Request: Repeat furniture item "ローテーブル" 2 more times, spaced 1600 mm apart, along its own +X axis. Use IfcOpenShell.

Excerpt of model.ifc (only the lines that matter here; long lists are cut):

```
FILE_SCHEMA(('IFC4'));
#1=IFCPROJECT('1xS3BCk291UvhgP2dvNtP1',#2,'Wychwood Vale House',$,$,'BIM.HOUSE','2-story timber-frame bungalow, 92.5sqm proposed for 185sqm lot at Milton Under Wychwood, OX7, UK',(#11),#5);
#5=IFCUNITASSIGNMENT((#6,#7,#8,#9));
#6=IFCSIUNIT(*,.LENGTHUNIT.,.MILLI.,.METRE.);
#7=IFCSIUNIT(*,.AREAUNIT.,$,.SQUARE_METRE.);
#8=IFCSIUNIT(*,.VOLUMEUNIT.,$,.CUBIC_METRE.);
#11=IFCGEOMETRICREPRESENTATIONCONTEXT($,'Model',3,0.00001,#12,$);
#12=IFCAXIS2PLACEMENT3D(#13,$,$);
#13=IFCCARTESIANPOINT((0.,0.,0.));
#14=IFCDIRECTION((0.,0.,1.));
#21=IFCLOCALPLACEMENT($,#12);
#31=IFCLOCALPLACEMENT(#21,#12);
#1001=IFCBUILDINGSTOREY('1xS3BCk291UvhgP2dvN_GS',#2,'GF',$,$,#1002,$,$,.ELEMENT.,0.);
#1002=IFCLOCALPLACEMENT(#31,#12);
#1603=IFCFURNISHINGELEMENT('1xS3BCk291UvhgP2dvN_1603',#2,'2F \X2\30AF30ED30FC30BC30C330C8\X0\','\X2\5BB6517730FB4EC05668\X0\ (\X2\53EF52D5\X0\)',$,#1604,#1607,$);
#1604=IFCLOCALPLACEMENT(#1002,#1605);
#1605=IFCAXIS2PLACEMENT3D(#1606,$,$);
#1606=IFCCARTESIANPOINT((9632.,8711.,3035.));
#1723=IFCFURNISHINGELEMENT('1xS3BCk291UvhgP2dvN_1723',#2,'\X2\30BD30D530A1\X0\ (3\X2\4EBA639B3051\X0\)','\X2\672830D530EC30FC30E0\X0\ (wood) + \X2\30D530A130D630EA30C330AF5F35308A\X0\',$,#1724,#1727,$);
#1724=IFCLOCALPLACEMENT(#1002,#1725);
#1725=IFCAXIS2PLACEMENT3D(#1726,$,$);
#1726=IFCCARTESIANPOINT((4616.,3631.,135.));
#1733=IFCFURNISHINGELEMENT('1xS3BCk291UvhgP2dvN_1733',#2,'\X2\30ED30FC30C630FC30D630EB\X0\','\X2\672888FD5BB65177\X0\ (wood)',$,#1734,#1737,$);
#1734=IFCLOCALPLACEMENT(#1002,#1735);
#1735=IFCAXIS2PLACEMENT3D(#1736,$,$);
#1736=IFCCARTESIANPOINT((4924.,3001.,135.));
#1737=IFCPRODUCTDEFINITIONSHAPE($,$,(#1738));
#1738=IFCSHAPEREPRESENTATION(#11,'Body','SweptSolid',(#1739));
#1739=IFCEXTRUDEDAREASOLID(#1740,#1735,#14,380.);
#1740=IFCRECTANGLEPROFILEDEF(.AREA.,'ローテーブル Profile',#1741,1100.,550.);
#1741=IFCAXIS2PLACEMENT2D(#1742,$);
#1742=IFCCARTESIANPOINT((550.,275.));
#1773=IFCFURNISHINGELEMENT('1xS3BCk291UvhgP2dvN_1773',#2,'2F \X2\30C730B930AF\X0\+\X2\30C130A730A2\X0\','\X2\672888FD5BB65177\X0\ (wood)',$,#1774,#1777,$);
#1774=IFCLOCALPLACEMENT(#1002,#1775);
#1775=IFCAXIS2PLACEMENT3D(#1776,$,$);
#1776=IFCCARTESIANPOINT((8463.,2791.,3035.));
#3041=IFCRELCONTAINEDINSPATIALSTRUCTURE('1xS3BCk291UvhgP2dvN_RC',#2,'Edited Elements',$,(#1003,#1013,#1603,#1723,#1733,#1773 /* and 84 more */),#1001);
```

```python
import ifcopenshell
import ifcopenshell.api.geometry
import ifcopenshell.api.root
import ifcopenshell.util.element
import ifcopenshell.util.placement

model = ifcopenshell.open("model.ifc")


def reuse_history(source, copy):
    """copy_class also copies each property set's owner history, people and application; keep the originals."""
    for rel in copy.IsDefinedBy:
        if rel.is_a("IfcRelDefinesByProperties") and (history := rel.RelatingPropertyDefinition.OwnerHistory):
            rel.RelatingPropertyDefinition.OwnerHistory = source.OwnerHistory
            ifcopenshell.util.element.remove_deep2(model, history)


source = model.by_guid("1xS3BCk291UvhgP2dvN_1733")
base = ifcopenshell.util.placement.get_local_placement(source.ObjectPlacement)
step = base[:3, 0] * 1600.0

for i in range(1, 3):
    copy = ifcopenshell.api.root.copy_class(model, product=source)
    copy.Representation = ifcopenshell.util.element.copy_deep(
        model, source.Representation, exclude=["IfcGeometricRepresentationContext", "IfcRepresentationMap"]
    )
    reuse_history(source, copy)
    matrix = base.copy()
    matrix[:3, 3] += i * step
    print("added at", matrix[:3, 3].round(3) + 0.0)
    ifcopenshell.api.geometry.edit_object_placement(model, product=copy, matrix=matrix, is_si=False)

model.write("model_v2.ifc")
```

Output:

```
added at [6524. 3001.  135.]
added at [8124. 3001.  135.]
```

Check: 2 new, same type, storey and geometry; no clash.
